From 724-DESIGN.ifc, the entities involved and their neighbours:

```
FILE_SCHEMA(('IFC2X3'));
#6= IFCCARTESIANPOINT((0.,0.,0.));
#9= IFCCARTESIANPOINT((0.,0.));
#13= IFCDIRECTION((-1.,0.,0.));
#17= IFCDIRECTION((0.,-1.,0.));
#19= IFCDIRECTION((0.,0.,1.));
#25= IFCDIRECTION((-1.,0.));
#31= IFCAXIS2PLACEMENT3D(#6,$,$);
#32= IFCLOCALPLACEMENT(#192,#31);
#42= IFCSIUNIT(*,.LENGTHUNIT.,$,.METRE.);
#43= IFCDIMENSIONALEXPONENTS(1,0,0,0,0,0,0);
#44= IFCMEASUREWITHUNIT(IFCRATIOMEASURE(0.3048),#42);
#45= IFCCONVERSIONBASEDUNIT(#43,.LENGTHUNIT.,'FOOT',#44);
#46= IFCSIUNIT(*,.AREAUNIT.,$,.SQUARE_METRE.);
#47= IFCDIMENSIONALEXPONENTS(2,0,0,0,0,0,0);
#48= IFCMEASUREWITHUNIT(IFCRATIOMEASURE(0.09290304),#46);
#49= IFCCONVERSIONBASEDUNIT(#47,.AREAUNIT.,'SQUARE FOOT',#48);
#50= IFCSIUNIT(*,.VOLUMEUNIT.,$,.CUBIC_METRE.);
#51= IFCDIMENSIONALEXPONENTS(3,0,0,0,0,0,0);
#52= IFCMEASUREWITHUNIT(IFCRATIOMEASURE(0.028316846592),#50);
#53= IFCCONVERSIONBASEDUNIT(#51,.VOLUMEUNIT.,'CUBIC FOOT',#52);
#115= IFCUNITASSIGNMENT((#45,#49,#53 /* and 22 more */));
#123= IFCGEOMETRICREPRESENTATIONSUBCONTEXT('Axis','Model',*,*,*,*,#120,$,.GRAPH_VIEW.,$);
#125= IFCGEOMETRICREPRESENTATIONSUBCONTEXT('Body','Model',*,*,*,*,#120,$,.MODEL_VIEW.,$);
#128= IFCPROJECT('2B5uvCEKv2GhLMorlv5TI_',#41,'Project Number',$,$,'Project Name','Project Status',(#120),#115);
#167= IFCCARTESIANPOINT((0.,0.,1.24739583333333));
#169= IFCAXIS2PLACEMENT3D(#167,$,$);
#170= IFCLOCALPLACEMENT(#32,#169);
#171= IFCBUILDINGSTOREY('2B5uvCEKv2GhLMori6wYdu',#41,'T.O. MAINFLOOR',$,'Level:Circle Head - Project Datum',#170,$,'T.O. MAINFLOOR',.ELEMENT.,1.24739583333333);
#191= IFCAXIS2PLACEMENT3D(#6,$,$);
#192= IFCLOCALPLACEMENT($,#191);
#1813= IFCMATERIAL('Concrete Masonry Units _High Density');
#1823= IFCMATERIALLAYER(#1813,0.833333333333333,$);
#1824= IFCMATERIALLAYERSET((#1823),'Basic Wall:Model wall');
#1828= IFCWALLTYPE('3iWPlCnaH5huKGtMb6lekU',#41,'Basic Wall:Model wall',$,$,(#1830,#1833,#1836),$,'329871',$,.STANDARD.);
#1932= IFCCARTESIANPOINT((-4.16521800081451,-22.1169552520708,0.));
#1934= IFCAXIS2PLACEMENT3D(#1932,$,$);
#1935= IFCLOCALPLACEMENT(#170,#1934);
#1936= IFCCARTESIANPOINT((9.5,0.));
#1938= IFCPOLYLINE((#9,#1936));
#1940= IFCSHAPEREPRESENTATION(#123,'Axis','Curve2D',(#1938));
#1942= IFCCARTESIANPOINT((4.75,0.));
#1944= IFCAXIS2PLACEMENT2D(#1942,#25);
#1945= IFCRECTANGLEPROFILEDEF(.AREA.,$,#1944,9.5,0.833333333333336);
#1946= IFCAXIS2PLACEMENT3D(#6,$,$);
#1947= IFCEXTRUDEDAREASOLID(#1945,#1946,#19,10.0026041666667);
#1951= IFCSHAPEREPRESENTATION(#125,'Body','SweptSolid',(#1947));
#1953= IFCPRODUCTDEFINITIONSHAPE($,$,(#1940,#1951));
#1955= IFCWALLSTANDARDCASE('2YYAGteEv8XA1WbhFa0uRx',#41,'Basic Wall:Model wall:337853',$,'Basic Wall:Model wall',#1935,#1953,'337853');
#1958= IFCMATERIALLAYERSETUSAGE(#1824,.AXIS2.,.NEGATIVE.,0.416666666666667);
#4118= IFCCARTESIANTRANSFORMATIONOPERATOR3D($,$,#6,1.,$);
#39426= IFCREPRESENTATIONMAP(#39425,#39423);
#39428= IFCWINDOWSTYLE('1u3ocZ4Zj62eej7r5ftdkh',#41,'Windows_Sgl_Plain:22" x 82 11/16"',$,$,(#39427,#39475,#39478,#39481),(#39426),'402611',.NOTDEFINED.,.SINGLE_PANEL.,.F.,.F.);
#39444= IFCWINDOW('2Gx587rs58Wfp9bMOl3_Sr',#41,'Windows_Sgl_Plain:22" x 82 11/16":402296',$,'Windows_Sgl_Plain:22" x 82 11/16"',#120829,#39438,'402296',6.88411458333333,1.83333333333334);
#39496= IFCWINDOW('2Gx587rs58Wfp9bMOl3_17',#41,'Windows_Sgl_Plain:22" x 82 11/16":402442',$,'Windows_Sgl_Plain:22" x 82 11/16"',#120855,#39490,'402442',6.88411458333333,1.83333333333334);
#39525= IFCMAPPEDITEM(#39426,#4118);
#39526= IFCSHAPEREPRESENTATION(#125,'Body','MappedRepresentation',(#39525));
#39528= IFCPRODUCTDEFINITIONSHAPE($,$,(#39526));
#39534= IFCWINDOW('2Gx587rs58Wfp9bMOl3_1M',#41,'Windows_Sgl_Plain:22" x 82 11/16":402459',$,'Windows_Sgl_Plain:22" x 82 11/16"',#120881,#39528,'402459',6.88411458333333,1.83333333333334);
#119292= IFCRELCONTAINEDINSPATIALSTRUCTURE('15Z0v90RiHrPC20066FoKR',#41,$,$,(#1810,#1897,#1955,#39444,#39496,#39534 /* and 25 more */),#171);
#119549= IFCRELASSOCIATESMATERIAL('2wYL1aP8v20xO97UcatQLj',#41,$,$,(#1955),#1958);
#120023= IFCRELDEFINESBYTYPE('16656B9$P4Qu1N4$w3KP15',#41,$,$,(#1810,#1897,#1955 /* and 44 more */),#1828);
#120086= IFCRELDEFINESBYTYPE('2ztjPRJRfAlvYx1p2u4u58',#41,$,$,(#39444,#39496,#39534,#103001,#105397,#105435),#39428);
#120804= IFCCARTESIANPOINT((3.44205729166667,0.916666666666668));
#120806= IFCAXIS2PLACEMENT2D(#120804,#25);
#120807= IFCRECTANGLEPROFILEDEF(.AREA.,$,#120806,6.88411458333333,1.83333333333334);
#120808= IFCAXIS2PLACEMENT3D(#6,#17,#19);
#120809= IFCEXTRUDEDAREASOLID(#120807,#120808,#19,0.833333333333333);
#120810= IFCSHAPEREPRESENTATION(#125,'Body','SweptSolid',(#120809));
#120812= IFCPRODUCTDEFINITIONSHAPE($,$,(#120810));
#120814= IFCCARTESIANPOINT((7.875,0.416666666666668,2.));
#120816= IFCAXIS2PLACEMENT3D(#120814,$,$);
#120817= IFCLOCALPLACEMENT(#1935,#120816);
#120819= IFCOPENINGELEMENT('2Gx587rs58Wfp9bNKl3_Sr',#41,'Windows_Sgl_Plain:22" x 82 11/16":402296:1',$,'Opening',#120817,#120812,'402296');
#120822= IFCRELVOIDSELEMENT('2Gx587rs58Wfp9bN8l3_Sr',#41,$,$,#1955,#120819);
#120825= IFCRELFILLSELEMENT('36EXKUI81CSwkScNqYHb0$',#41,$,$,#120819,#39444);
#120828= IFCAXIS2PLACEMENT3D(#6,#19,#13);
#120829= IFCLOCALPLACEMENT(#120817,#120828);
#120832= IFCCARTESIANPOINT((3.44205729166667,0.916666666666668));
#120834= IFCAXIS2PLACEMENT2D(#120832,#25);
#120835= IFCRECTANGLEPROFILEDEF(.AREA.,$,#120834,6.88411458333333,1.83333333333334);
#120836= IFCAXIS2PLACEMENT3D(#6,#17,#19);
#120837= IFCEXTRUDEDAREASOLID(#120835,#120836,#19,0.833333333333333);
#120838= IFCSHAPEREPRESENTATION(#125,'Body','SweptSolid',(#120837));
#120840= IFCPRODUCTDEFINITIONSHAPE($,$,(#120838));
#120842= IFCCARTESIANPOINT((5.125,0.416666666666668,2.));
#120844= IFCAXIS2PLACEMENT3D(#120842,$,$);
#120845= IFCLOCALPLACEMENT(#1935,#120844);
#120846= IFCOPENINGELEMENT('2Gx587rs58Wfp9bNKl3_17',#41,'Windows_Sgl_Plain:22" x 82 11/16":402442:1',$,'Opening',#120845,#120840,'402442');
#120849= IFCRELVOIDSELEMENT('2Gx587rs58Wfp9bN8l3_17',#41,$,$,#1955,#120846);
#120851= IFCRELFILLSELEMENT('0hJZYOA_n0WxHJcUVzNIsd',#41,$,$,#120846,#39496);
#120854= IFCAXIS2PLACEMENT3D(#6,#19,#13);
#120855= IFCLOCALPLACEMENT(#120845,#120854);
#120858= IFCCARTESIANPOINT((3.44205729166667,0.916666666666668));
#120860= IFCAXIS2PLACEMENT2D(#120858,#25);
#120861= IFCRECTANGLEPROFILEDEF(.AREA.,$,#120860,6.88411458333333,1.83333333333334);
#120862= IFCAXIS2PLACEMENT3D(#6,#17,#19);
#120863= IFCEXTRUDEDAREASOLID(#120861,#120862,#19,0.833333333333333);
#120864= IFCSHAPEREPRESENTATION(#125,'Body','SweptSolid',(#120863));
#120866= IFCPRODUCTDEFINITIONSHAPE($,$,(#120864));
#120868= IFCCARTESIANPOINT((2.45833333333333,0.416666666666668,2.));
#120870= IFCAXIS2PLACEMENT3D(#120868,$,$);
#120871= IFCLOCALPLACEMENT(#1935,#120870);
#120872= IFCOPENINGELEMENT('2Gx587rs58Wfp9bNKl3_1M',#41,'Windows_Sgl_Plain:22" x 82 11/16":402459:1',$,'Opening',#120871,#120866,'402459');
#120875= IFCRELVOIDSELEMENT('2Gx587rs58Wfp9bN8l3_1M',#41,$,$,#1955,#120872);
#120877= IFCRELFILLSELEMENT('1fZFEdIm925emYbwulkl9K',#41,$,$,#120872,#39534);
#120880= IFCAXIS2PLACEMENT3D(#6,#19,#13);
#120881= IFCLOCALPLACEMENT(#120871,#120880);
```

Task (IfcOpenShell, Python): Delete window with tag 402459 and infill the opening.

```python
import ifcopenshell
import ifcopenshell.api.feature
import ifcopenshell.api.root
import ifcopenshell.geom
import ifcopenshell.util.shape

model = ifcopenshell.open("724-DESIGN.ifc")
settings = ifcopenshell.geom.settings()


def volume(element):
    """Net volume in cubic metres, openings subtracted."""
    shape = ifcopenshell.geom.create_shape(settings, element)
    return ifcopenshell.util.shape.get_volume(shape.geometry)


window = model.by_guid("2Gx587rs58Wfp9bMOl3_1M")
opening = window.FillsVoids[0].RelatingOpeningElement
wall = opening.VoidsElements[0].RelatingBuildingElement
before = volume(wall)

ifcopenshell.api.root.remove_product(model, product=window)
ifcopenshell.api.feature.remove_feature(model, feature=opening)

after = volume(wall)

print(f"wall volume {before:.3f} -> {after:.3f} m3")

model.write("724-DESIGN_rev.ifc")
```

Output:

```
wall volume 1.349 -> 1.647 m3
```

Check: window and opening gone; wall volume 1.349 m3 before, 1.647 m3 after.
